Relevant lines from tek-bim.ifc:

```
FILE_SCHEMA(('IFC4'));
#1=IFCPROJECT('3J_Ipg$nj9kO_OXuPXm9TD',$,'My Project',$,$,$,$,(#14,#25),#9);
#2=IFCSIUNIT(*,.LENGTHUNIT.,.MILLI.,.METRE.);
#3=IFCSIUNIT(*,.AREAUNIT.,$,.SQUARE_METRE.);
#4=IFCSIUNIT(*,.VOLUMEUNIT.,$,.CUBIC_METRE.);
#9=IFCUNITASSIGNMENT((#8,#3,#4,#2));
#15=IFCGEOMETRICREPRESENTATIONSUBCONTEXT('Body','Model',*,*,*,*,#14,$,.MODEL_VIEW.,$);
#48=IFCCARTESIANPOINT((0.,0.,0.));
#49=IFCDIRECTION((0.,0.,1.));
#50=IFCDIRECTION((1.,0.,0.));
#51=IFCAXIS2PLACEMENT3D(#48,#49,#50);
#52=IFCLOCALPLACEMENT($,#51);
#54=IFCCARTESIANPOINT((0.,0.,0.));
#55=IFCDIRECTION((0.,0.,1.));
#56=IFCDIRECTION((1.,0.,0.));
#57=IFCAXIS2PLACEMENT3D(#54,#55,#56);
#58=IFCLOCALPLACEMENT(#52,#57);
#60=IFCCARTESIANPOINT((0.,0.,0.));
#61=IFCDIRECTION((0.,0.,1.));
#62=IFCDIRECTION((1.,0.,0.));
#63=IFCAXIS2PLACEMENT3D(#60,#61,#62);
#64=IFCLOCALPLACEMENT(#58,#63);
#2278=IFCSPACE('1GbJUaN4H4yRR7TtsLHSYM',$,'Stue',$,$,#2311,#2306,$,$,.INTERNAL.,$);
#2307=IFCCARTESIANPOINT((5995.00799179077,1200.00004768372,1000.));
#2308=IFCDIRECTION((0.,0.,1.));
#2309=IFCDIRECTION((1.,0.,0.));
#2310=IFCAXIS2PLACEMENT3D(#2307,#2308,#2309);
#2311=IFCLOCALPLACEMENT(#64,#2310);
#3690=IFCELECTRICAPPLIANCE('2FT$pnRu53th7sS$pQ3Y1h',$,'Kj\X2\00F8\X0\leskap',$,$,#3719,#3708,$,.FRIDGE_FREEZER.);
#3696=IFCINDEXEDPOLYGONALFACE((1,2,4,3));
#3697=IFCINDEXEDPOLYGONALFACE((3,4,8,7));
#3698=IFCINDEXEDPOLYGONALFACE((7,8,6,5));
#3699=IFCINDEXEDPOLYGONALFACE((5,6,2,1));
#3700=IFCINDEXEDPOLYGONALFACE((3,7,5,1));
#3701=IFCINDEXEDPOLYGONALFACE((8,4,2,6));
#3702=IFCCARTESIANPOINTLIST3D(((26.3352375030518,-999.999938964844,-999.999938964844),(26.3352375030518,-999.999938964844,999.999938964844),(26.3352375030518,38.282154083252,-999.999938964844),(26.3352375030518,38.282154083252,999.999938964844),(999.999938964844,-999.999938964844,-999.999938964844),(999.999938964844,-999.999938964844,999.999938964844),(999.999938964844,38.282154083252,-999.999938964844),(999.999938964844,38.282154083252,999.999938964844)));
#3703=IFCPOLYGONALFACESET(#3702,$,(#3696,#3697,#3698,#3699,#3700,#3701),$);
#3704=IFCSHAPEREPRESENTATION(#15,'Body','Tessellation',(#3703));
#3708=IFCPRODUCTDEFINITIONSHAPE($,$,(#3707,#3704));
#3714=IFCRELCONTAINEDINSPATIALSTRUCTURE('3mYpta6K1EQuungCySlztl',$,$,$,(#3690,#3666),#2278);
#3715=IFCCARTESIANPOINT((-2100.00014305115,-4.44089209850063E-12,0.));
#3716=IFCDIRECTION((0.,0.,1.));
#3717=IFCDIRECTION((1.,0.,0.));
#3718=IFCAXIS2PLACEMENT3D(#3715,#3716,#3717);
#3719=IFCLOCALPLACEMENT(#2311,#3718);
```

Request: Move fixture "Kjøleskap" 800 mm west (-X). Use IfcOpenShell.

```python
import ifcopenshell
import ifcopenshell.api.geometry
import ifcopenshell.util.placement
import ifcopenshell.util.unit

model = ifcopenshell.open("tek-bim.ifc")
unit_scale = ifcopenshell.util.unit.calculate_unit_scale(model)

item = model.by_guid("2FT$pnRu53th7sS$pQ3Y1h")
matrix = ifcopenshell.util.placement.get_local_placement(item.ObjectPlacement)
matrix[0, 3] -= 0.8 / unit_scale
ifcopenshell.api.geometry.edit_object_placement(model, product=item, matrix=matrix, is_si=False)

print(ifcopenshell.util.placement.get_local_placement(item.ObjectPlacement).round(3) + 0.0)

model.write("tek-bim_rev.ifc")
```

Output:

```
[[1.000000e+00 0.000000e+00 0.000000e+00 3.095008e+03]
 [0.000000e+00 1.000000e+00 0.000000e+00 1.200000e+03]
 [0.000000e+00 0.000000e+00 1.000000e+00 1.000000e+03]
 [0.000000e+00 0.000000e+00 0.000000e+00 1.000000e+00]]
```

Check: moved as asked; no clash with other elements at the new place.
